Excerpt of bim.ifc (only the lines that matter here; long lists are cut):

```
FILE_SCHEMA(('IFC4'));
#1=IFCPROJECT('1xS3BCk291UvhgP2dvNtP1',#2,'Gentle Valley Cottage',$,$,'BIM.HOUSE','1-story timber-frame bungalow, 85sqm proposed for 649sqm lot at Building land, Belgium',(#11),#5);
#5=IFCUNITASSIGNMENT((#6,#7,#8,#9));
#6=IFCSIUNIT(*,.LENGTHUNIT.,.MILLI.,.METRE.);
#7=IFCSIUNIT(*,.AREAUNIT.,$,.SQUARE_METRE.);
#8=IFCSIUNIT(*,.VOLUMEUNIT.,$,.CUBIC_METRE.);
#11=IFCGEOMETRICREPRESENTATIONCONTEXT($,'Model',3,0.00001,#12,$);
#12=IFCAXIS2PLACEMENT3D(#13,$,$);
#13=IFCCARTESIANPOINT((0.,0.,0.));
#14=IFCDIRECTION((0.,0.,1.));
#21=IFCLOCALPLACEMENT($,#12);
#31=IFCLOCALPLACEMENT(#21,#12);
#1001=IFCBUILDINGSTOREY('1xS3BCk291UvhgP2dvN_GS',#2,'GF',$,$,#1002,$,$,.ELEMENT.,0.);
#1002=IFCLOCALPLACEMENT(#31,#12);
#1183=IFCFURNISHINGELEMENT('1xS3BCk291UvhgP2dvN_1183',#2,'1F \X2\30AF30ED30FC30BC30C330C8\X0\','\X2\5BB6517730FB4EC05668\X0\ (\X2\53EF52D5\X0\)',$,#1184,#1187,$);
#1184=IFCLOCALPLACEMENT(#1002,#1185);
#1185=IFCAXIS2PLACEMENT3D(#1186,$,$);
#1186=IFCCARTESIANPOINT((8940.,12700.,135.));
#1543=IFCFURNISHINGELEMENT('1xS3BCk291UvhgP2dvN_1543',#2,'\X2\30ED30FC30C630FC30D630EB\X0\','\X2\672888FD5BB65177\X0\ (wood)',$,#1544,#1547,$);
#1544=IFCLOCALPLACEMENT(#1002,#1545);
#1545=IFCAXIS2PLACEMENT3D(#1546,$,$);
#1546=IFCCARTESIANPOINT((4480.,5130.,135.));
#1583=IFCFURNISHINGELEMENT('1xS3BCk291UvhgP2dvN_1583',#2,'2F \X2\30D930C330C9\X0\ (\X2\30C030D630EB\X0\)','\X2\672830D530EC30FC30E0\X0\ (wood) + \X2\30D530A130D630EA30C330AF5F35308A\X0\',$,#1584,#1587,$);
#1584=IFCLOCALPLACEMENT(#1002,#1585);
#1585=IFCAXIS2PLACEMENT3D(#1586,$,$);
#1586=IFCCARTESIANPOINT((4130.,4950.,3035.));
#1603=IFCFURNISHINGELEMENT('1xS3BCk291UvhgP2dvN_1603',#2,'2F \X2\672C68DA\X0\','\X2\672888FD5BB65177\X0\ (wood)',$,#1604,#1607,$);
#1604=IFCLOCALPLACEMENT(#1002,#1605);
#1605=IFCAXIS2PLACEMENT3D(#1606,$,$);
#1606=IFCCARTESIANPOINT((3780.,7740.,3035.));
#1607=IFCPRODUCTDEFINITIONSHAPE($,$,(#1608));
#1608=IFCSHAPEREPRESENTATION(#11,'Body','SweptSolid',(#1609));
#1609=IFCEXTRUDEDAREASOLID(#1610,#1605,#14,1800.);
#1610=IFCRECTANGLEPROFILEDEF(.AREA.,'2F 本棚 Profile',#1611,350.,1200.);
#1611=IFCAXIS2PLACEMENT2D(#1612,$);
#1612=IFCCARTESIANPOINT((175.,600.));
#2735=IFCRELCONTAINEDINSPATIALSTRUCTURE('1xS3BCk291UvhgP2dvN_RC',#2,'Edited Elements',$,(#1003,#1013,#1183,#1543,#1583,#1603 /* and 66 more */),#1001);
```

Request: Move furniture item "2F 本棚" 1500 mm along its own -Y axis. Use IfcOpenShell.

```python
import ifcopenshell
import ifcopenshell.api.geometry
import ifcopenshell.util.placement
import ifcopenshell.util.unit

model = ifcopenshell.open("bim.ifc")
unit_scale = ifcopenshell.util.unit.calculate_unit_scale(model)

item = model.by_guid("1xS3BCk291UvhgP2dvN_1603")
matrix = ifcopenshell.util.placement.get_local_placement(item.ObjectPlacement)
matrix[:3, 3] -= matrix[:3, 1] * 1.5 / unit_scale
ifcopenshell.api.geometry.edit_object_placement(model, product=item, matrix=matrix, is_si=False)

print(ifcopenshell.util.placement.get_local_placement(item.ObjectPlacement).round(3) + 0.0)

model.write("bim-out.ifc")
```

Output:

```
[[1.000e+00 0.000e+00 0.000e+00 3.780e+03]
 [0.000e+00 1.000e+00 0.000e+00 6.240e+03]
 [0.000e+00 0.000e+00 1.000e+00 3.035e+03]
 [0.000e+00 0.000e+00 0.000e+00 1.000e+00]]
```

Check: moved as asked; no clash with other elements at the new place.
